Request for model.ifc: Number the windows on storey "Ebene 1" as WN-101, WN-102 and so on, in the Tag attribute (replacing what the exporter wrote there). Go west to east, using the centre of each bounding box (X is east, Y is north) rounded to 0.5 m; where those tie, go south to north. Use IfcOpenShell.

First a look at what the model holds.

```python
import ifcopenshell
import ifcopenshell.util.element
import ifcopenshell.util.placement

model = ifcopenshell.open("model.ifc")
print(model.schema)
storey = next(s for s in model.by_type("IfcBuildingStorey") if s.Name == "Ebene 1")
windows = [e for e in ifcopenshell.util.element.get_decomposition(storey) if e.is_a("IfcWindow")]
for e in sorted(windows, key=lambda e: e.id()):
    origin = ifcopenshell.util.placement.get_local_placement(e.ObjectPlacement)[:3, 3]
    print(e.id(), e.Tag, e.Name, origin.round(2) + 0.0, sep=" | ")
```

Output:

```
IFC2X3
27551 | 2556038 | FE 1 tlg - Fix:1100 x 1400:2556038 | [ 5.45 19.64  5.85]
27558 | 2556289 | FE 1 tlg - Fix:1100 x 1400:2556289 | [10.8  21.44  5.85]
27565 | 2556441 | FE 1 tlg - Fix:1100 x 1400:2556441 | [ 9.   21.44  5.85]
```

```python
import ifcopenshell
import ifcopenshell.geom
import ifcopenshell.util.element
import ifcopenshell.util.shape

model = ifcopenshell.open("model.ifc")
settings = ifcopenshell.geom.settings()
settings.set("use-world-coords", True)


def centre(element):
    shape = ifcopenshell.geom.create_shape(settings, element)
    return ifcopenshell.util.shape.get_bbox_centroid(shape.geometry)


storey = next(s for s in model.by_type("IfcBuildingStorey") if s.Name == "Ebene 1")
windows = [e for e in ifcopenshell.util.element.get_decomposition(storey) if e.is_a("IfcWindow")]

# Insertion points can sit at a corner or the storey origin, so sort by the geometry (in metres).
centres = {e: centre(e) for e in windows}
windows.sort(key=lambda e: (round(centres[e][0] / 0.5), centres[e][1]))

for i, e in enumerate(windows, start=1):
    number = f"WN-1{i:02d}"
    e.Tag = number
    print(e.id(), number)

model.write("model_updated.ifc")
```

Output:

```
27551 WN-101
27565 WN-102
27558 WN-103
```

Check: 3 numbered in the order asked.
